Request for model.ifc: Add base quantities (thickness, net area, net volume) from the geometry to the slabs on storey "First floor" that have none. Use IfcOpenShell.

First a look at what the model holds.

```python
import ifcopenshell
import ifcopenshell.util.element
import ifcopenshell.util.unit

model = ifcopenshell.open("model.ifc")
print(model.schema)
for unit_type in ("LENGTHUNIT", "AREAUNIT", "VOLUMEUNIT"):
    print(unit_type, ifcopenshell.util.unit.calculate_unit_scale(model, unit_type))
storey = next(s for s in model.by_type("IfcBuildingStorey") if s.Name == "First floor")
slabs = [e for e in ifcopenshell.util.element.get_decomposition(storey) if e.is_a("IfcSlab")]
for e in sorted(slabs, key=lambda e: e.id()):
    print(e.id(), e.is_a(), e.Name, list(ifcopenshell.util.element.get_psets(e, qtos_only=True)), sep=" | ")
```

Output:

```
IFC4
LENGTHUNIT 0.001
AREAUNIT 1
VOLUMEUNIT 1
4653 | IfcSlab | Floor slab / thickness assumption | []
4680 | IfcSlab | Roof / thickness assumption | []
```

```python
import ifcopenshell
import ifcopenshell.api.pset
import ifcopenshell.geom
import ifcopenshell.util.element
import ifcopenshell.util.shape
import ifcopenshell.util.unit

model = ifcopenshell.open("model.ifc")
unit_scale = ifcopenshell.util.unit.calculate_unit_scale(model)
area_scale = ifcopenshell.util.unit.calculate_unit_scale(model, "AREAUNIT")
volume_scale = ifcopenshell.util.unit.calculate_unit_scale(model, "VOLUMEUNIT")
settings = ifcopenshell.geom.settings()

storey = next(s for s in model.by_type("IfcBuildingStorey") if s.Name == "First floor")
slabs = [e for e in ifcopenshell.util.element.get_decomposition(storey) if e.is_a("IfcSlab")]

for e in sorted(slabs, key=lambda e: e.id()):
    if ifcopenshell.util.element.get_psets(e, qtos_only=True, should_inherit=False):
        continue
    # Geometry comes back in metres, in the element's own axes.
    shape = ifcopenshell.geom.create_shape(settings, e)
    values = {
        "Width": ifcopenshell.util.shape.get_z(shape.geometry) / unit_scale,
        "NetArea": ifcopenshell.util.shape.get_footprint_area(shape.geometry) / area_scale,
        "NetVolume": ifcopenshell.util.shape.get_volume(shape.geometry) / volume_scale,
    }
    qto = ifcopenshell.api.pset.add_qto(model, product=e, name="Qto_SlabBaseQuantities")
    ifcopenshell.api.pset.edit_qto(model, qto=qto, properties=values)
    print(e.id(), {k: round(v, 3) for k, v in values.items()})

model.write("model_updated.ifc")
```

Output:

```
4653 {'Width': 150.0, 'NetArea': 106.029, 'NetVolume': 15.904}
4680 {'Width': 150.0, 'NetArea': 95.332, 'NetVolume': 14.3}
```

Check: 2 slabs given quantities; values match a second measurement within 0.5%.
